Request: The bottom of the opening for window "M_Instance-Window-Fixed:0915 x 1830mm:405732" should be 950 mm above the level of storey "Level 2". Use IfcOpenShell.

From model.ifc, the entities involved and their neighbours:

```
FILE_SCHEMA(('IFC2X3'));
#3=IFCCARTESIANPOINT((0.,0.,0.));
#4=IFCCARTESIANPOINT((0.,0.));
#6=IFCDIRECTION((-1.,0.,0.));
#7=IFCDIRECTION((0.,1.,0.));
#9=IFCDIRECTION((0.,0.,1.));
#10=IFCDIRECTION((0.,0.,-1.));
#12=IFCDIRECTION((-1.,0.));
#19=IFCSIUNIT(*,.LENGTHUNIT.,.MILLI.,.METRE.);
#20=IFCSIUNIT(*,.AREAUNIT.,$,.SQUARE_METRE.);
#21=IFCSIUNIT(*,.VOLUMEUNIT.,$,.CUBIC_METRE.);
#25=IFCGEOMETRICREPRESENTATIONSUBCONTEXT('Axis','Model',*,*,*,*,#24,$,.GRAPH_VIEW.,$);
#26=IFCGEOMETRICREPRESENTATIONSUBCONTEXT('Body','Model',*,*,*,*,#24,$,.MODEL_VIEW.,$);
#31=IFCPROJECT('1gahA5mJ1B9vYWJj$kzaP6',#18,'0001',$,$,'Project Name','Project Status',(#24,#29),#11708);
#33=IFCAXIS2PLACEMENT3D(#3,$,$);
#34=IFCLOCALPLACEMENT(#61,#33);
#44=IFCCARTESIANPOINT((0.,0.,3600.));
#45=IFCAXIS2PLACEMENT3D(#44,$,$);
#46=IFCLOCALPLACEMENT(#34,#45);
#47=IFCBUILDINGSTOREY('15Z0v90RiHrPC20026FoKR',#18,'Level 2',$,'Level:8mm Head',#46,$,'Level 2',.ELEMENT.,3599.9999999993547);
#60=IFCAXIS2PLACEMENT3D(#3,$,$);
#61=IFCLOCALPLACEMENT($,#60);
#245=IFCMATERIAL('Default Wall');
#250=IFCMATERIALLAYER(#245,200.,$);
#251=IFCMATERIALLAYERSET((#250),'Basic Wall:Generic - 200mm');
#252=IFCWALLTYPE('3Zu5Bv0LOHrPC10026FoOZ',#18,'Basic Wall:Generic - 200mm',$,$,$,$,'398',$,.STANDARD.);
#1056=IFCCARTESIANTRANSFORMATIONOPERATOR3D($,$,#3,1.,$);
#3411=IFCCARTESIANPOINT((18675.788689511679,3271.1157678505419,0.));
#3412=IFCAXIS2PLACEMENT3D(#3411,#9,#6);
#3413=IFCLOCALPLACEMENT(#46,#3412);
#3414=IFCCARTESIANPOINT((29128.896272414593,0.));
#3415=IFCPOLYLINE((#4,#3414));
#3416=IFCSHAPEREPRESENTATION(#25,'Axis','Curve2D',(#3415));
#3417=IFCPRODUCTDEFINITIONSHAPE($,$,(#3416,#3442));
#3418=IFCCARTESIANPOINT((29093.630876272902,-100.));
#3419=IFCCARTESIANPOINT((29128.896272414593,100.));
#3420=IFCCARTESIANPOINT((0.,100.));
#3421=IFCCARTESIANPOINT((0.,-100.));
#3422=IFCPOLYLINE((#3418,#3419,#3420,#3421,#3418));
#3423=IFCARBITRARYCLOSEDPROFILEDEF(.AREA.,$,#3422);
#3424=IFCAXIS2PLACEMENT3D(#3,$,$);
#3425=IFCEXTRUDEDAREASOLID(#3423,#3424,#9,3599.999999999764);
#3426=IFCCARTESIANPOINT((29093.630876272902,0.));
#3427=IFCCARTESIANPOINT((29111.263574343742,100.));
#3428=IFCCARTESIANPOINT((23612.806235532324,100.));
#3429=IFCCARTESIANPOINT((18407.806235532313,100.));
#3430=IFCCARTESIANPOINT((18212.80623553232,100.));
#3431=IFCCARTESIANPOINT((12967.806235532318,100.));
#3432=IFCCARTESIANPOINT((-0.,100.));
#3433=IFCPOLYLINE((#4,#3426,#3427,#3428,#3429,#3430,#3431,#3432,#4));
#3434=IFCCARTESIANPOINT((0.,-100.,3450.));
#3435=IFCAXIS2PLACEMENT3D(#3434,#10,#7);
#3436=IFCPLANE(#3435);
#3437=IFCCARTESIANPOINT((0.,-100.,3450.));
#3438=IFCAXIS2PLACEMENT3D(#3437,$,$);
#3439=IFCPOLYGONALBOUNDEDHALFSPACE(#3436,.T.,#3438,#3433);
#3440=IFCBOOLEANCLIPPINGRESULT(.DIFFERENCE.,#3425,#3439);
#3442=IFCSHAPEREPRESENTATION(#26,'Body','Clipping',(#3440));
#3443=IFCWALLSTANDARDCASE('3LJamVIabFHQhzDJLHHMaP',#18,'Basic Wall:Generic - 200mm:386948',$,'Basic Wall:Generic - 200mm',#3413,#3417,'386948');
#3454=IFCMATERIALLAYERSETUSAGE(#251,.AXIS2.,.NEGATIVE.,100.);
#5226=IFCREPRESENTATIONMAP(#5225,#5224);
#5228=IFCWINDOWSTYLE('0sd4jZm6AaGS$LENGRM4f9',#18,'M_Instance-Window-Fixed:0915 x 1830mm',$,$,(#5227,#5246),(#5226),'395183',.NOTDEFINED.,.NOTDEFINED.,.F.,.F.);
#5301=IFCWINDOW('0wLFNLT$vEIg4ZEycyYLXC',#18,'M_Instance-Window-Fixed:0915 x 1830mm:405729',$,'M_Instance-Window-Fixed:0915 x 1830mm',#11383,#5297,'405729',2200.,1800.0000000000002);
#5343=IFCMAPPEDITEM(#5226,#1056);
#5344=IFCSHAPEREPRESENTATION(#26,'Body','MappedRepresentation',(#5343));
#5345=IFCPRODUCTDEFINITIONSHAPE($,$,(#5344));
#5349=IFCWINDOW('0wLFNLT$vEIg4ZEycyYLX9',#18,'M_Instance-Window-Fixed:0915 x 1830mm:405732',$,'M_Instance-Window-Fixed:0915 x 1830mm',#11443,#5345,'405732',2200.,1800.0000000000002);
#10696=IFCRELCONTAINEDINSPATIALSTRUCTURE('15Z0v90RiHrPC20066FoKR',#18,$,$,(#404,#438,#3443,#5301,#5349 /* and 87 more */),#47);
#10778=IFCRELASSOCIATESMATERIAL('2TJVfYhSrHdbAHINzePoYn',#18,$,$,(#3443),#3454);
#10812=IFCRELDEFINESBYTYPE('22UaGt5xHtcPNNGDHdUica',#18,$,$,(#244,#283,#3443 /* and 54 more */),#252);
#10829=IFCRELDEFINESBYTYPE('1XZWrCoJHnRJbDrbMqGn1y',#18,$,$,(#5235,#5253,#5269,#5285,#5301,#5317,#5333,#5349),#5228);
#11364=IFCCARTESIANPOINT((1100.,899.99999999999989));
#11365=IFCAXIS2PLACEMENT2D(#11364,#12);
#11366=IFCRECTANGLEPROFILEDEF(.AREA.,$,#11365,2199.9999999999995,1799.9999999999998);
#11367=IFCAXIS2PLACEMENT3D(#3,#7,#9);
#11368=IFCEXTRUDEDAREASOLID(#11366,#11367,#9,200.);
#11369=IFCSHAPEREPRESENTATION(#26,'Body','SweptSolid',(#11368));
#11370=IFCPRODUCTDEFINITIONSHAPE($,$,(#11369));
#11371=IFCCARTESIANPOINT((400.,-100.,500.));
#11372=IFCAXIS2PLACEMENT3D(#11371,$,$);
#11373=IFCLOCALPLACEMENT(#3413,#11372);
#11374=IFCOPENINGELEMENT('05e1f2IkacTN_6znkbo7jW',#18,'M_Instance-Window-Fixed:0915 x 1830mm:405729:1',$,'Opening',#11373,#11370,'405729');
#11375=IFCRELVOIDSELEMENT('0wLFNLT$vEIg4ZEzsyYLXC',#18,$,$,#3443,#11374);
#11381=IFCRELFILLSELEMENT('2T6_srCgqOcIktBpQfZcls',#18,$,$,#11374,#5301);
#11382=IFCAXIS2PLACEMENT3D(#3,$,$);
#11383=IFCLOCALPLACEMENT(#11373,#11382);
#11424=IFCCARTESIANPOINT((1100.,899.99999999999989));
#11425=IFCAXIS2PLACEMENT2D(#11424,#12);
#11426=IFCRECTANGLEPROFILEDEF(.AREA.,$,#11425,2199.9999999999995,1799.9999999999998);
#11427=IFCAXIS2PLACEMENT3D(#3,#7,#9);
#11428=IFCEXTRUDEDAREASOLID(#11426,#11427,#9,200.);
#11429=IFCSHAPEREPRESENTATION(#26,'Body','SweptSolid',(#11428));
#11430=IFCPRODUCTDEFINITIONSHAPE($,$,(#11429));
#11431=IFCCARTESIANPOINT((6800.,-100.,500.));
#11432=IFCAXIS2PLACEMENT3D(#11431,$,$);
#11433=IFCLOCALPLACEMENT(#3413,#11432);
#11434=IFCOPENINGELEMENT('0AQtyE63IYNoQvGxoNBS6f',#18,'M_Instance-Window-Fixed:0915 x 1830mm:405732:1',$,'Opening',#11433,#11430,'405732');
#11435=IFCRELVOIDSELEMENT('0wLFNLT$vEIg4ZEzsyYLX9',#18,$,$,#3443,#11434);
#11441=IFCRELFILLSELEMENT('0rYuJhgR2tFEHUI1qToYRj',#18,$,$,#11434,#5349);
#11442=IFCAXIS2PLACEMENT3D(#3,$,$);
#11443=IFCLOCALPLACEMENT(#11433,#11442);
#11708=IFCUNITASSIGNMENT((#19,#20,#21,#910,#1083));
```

```python
import numpy as np
import ifcopenshell
import ifcopenshell.api.geometry
import ifcopenshell.geom
import ifcopenshell.util.element
import ifcopenshell.util.placement
import ifcopenshell.util.shape
import ifcopenshell.util.unit

model = ifcopenshell.open("model.ifc")
unit_scale = ifcopenshell.util.unit.calculate_unit_scale(model)

window = model.by_id(5349)
opening = window.FillsVoids[0].RelatingOpeningElement
storey = ifcopenshell.util.element.get_container(window, ifc_class="IfcBuildingStorey")
level = ifcopenshell.util.placement.get_local_placement(storey.ObjectPlacement)[2, 3]

# The opening's origin need not be at the sill, so measure its lowest point.
shape = ifcopenshell.geom.create_shape(ifcopenshell.geom.settings(), opening)
bottom = ifcopenshell.util.shape.get_shape_bottom_elevation(shape, shape.geometry) / unit_scale
dz = level + 0.95 / unit_scale - bottom

shift = np.array([0.0, 0.0, dz])
# The window is placed relative to its opening, so it follows when the opening moves.
matrix = ifcopenshell.util.placement.get_local_placement(opening.ObjectPlacement)
matrix[:3, 3] += shift
ifcopenshell.api.geometry.edit_object_placement(
    model, product=opening, matrix=matrix, is_si=False, should_transform_children=True
)

print(f"moved by {dz * unit_scale:+.3f} m")

model.write("model_updated.ifc")
```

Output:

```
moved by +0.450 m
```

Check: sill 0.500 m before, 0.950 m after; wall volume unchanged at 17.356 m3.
